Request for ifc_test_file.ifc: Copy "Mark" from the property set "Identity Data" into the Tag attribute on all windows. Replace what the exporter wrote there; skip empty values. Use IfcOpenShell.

First a look at what the model holds.

```python
import ifcopenshell
import ifcopenshell.util.element

model = ifcopenshell.open("ifc_test_file.ifc")
print(model.schema)
windows = model.by_type("IfcWindow")
print(len(windows), "windows")
for e in windows[:8]:
    source = ifcopenshell.util.element.get_pset(e, "Identity Data", "Mark")
    target = e.Tag
    print(e.id(), repr(source), repr(target), sep=" | ")
```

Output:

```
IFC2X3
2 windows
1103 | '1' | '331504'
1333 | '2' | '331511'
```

```python
import ifcopenshell
import ifcopenshell.util.element

model = ifcopenshell.open("ifc_test_file.ifc")

count = 0
for e in model.by_type("IfcWindow"):
    value = ifcopenshell.util.element.get_pset(e, "Identity Data", "Mark")
    current = e.Tag
    if not value or not value.strip() or current == value:
        continue
    e.Tag = value
    count += 1

print(count, "windows updated")

model.write("ifc_test_file-out.ifc")
```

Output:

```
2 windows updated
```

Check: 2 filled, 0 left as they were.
